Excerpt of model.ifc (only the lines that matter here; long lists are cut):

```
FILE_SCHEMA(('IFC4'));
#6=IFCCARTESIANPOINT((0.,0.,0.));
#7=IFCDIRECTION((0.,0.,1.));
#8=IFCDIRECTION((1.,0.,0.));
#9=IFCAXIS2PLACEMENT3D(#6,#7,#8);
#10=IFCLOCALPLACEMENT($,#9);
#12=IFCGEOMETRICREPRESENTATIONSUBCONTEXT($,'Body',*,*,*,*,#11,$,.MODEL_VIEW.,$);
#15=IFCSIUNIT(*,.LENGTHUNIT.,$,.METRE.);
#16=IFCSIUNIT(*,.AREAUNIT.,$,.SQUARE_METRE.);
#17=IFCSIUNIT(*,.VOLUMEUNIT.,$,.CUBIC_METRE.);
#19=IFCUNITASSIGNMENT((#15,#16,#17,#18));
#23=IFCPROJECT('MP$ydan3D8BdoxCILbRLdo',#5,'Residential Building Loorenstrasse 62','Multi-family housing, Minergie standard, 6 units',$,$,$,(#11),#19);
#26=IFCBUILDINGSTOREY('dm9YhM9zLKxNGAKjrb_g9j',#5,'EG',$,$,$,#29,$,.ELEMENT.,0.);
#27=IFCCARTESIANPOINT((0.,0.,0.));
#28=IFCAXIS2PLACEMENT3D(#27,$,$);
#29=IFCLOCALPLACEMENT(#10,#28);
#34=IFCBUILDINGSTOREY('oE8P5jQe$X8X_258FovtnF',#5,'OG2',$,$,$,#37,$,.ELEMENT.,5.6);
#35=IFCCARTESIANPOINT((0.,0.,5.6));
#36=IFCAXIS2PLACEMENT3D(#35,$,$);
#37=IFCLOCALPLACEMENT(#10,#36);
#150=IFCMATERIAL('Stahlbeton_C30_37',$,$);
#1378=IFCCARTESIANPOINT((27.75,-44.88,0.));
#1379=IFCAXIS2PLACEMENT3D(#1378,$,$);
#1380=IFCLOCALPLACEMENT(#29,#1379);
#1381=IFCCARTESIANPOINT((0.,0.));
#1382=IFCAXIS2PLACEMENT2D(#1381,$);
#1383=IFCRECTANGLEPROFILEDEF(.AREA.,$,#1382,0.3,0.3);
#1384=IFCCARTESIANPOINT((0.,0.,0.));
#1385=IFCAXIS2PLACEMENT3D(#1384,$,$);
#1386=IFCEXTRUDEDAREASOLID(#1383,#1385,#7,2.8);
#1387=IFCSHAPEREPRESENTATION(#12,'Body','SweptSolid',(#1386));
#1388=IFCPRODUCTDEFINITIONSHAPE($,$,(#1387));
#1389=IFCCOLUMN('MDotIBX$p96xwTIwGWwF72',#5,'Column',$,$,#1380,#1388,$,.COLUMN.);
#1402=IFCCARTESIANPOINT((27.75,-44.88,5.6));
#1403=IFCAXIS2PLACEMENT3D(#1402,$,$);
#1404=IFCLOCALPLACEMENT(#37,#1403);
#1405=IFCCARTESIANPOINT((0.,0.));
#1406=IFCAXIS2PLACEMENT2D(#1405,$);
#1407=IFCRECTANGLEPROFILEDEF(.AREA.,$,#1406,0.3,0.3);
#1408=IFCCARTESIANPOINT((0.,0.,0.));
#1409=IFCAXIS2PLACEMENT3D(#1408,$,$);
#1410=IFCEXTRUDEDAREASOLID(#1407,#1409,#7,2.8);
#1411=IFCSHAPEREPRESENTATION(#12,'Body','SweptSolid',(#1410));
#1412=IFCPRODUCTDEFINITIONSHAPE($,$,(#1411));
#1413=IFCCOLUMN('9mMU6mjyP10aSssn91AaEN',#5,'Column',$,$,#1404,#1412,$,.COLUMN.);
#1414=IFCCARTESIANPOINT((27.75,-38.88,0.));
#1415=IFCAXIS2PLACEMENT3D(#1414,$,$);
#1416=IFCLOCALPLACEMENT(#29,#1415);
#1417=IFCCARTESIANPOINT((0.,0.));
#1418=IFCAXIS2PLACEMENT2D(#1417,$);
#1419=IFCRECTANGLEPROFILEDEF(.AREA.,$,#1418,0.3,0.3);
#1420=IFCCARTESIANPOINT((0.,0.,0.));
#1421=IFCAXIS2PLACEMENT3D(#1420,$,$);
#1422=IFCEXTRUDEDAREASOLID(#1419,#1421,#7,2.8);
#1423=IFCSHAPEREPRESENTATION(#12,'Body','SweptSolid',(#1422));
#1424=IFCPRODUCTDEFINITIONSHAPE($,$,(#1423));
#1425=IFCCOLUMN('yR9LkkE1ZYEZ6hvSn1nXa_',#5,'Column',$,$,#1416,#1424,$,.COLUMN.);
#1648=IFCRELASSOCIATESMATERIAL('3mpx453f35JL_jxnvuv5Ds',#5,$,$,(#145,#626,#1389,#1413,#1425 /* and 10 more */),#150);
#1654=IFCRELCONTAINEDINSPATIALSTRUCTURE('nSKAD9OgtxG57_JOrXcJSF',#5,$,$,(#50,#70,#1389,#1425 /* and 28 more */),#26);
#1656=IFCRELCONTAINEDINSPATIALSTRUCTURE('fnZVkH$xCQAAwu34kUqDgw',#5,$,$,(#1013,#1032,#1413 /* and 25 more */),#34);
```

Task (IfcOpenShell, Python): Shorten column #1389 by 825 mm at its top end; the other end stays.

```python
import ifcopenshell
import ifcopenshell.util.unit

model = ifcopenshell.open("model.ifc")
unit_scale = ifcopenshell.util.unit.calculate_unit_scale(model)

member = model.by_id(1389)
change = -0.825 / unit_scale

# The extrusion runs towards the end named, so only its depth changes.
body = next(r for r in member.Representation.Representations if r.RepresentationIdentifier == "Body")
solid = body.Items[0]
old_length = solid.Depth
solid.Depth += change

print(f"length {old_length:g} -> {solid.Depth:g}")

model.write("model_rev.ifc")
```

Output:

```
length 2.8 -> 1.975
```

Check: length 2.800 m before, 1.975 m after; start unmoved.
